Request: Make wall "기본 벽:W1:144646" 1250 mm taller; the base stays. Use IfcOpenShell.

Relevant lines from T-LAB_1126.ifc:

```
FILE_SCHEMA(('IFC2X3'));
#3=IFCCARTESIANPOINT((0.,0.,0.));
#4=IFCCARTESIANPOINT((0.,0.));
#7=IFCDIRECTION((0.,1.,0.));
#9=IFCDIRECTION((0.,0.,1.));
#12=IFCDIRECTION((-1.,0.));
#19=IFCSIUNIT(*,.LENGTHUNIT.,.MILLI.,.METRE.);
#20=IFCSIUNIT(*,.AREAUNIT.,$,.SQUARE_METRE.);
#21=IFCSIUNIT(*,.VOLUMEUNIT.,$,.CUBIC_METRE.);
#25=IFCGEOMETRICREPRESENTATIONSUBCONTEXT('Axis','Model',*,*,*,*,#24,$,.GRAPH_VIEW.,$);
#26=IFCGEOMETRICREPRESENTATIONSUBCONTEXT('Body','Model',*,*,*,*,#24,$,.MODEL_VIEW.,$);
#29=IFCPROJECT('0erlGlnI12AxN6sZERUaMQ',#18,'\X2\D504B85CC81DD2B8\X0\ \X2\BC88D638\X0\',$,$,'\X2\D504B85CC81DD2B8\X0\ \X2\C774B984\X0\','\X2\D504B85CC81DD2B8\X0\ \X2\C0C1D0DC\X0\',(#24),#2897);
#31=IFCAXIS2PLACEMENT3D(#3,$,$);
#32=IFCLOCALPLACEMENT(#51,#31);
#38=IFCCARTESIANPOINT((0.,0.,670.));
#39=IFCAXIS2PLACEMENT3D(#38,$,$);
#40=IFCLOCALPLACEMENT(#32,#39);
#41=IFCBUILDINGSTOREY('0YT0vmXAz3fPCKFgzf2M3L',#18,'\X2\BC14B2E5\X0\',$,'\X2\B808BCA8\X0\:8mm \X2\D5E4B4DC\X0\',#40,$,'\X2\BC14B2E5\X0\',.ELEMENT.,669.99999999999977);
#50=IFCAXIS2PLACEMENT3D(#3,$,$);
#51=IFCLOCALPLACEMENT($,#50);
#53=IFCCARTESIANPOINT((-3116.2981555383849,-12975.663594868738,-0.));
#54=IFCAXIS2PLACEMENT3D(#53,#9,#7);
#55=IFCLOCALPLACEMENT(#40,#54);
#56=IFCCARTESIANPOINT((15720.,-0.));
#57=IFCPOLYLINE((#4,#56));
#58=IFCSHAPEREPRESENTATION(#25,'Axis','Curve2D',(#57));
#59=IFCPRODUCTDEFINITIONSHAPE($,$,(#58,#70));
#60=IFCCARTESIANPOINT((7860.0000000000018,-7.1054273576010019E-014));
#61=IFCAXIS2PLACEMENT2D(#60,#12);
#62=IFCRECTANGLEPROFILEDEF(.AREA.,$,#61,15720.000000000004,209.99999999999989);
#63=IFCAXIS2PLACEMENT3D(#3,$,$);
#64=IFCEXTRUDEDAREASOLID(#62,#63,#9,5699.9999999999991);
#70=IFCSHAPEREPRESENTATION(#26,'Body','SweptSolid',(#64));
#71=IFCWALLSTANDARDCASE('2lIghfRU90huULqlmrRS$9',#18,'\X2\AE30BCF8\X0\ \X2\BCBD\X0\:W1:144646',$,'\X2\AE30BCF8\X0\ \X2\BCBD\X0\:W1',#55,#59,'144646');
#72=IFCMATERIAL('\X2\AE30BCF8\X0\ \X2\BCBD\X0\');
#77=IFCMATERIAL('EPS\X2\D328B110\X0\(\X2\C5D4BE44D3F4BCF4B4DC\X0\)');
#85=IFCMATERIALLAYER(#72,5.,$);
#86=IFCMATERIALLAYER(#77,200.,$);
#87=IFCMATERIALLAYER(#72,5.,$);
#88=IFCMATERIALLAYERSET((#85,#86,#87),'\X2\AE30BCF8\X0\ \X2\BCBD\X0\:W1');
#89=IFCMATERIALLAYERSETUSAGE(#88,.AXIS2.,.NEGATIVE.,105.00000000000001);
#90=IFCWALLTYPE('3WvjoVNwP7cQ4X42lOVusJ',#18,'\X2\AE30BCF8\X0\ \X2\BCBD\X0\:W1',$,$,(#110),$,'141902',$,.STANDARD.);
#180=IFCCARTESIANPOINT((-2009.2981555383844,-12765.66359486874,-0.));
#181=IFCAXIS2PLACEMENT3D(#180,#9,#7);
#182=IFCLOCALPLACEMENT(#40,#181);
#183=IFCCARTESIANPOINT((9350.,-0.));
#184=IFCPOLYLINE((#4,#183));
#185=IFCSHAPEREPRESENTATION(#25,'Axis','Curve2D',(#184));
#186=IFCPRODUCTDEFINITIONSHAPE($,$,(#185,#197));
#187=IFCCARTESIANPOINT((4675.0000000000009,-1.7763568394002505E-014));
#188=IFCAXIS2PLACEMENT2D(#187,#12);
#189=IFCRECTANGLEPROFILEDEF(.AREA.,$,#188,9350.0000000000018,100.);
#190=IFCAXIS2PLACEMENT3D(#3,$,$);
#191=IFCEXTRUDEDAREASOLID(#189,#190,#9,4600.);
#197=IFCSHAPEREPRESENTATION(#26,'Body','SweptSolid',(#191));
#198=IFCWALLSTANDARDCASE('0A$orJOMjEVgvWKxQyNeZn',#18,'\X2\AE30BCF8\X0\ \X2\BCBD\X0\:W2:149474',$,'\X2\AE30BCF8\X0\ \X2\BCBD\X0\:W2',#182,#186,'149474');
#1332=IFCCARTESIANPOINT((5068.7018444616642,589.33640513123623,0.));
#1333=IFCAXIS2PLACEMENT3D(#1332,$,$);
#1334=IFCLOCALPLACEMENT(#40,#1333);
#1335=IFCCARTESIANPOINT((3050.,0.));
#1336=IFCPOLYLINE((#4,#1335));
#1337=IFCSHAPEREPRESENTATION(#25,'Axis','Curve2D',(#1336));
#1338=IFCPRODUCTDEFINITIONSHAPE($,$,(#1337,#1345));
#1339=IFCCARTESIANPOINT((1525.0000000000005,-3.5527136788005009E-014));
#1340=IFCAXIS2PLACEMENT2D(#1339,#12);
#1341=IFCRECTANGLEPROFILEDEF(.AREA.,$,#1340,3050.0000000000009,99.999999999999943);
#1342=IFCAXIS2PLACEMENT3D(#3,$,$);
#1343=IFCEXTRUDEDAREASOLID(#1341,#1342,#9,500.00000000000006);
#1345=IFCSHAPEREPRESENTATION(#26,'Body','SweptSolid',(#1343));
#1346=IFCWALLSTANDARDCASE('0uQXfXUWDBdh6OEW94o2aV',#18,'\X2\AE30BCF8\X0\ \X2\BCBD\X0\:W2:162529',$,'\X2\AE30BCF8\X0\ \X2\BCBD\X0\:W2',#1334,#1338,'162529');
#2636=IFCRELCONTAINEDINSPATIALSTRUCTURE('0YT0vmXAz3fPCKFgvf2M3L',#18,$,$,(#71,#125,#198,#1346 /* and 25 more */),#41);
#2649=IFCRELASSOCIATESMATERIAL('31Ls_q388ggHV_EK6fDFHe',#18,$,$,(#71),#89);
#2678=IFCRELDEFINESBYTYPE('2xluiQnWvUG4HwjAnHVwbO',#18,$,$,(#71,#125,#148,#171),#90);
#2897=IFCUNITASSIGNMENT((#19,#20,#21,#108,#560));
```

```python
import ifcopenshell
import ifcopenshell.geom
import ifcopenshell.util.representation
import ifcopenshell.util.shape

model = ifcopenshell.open("T-LAB_1126.ifc")
settings = ifcopenshell.geom.settings()


def volume(element):
    """Net volume in cubic metres, openings subtracted."""
    shape = ifcopenshell.geom.create_shape(settings, element)
    return ifcopenshell.util.shape.get_volume(shape.geometry)


wall = model.by_guid("2lIghfRU90huULqlmrRS$9")
before = volume(wall)

body = ifcopenshell.util.representation.get_representation(wall, "Model", "Body")
solid = body.Items[0]
old_height = solid.Depth
solid.Depth += 1250.0
after = volume(wall)

print(f"height {old_height:g} -> {solid.Depth:g}, volume {before:.3f} -> {after:.3f} m3")

model.write("T-LAB_1126_updated.ifc")
```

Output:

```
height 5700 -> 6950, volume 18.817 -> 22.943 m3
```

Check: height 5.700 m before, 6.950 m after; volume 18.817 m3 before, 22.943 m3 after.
